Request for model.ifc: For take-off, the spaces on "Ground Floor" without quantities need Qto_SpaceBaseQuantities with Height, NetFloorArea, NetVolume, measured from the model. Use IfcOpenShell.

First a look at what the model holds.

```python
import ifcopenshell
import ifcopenshell.util.element
import ifcopenshell.util.unit

model = ifcopenshell.open("model.ifc")
print(model.schema)
for unit_type in ("LENGTHUNIT", "AREAUNIT", "VOLUMEUNIT"):
    print(unit_type, ifcopenshell.util.unit.calculate_unit_scale(model, unit_type))
storey = next(s for s in model.by_type("IfcBuildingStorey") if s.Name == "Ground Floor")
spaces = [e for e in ifcopenshell.util.element.get_decomposition(storey) if e.is_a("IfcSpace")]
for e in sorted(spaces, key=lambda e: e.id()):
    print(e.id(), e.is_a(), e.Name, list(ifcopenshell.util.element.get_psets(e, qtos_only=True)), sep=" | ")
```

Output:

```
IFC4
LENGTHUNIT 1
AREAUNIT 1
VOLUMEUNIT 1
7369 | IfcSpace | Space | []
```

```python
import ifcopenshell
import ifcopenshell.api.pset
import ifcopenshell.geom
import ifcopenshell.util.element
import ifcopenshell.util.shape
import ifcopenshell.util.unit

model = ifcopenshell.open("model.ifc")
unit_scale = ifcopenshell.util.unit.calculate_unit_scale(model)
area_scale = ifcopenshell.util.unit.calculate_unit_scale(model, "AREAUNIT")
volume_scale = ifcopenshell.util.unit.calculate_unit_scale(model, "VOLUMEUNIT")
settings = ifcopenshell.geom.settings()

storey = next(s for s in model.by_type("IfcBuildingStorey") if s.Name == "Ground Floor")
spaces = [e for e in ifcopenshell.util.element.get_decomposition(storey) if e.is_a("IfcSpace")]

for e in sorted(spaces, key=lambda e: e.id()):
    if ifcopenshell.util.element.get_psets(e, qtos_only=True, should_inherit=False):
        continue
    # Geometry comes back in metres, in the element's own axes.
    shape = ifcopenshell.geom.create_shape(settings, e)
    values = {
        "Height": ifcopenshell.util.shape.get_z(shape.geometry) / unit_scale,
        "NetFloorArea": ifcopenshell.util.shape.get_footprint_area(shape.geometry) / area_scale,
        "NetVolume": ifcopenshell.util.shape.get_volume(shape.geometry) / volume_scale,
    }
    qto = ifcopenshell.api.pset.add_qto(model, product=e, name="Qto_SpaceBaseQuantities")
    ifcopenshell.api.pset.edit_qto(model, qto=qto, properties=values)
    print(e.id(), {k: round(v, 3) for k, v in values.items()})

model.write("model_v2.ifc")
```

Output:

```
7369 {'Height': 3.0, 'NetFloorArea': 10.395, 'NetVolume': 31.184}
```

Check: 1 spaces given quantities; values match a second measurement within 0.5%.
